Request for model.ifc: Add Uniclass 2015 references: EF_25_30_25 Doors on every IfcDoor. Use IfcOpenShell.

First a look at what the model holds.

```python
import ifcopenshell

model = ifcopenshell.open("model.ifc")
print(model.schema)
print("classifications:", [c.Name for c in model.by_type("IfcClassification")])
for ifc_class in ("IfcDoor", "IfcRoof", "IfcStair", "IfcWall", "IfcWindow"):
    print(ifc_class, len(model.by_type(ifc_class)))
```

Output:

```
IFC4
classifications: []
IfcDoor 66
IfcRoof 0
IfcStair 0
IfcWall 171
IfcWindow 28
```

```python
import ifcopenshell
import ifcopenshell.api.classification

model = ifcopenshell.open("model.ifc")

system = ifcopenshell.api.classification.add_classification(model, classification="Uniclass 2015")

codes = {
    "IfcDoor": ("EF_25_30_25", "Doors"),
}
for ifc_class, (code, name) in codes.items():
    products = model.by_type(ifc_class)
    ifcopenshell.api.classification.add_reference(
        model, products=products, classification=system, identification=code, name=name
    )
    print(code, len(products))

model.write("model_v2.ifc")
```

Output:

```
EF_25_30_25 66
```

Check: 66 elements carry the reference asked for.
